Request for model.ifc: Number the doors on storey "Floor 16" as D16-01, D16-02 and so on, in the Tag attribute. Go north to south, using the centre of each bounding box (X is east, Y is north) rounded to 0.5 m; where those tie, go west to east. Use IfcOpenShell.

First a look at what the model holds.

```python
import ifcopenshell
import ifcopenshell.util.element
import ifcopenshell.util.placement

model = ifcopenshell.open("model.ifc")
print(model.schema)
storey = next(s for s in model.by_type("IfcBuildingStorey") if s.Name == "Floor 16")
doors = [e for e in ifcopenshell.util.element.get_decomposition(storey) if e.is_a("IfcDoor")]
for e in sorted(doors, key=lambda e: e.id()):
    origin = ifcopenshell.util.placement.get_local_placement(e.ObjectPlacement)[:3, 3]
    print(e.id(), e.Tag, e.Name, origin.round(2) + 0.0, sep=" | ")
```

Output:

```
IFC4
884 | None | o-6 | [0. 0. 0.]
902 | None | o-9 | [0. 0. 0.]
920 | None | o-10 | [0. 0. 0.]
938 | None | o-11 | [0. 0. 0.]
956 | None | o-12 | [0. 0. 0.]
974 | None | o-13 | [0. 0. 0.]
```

```python
import ifcopenshell
import ifcopenshell.geom
import ifcopenshell.util.element
import ifcopenshell.util.shape

model = ifcopenshell.open("model.ifc")
settings = ifcopenshell.geom.settings()
settings.set("use-world-coords", True)


def centre(element):
    shape = ifcopenshell.geom.create_shape(settings, element)
    return ifcopenshell.util.shape.get_bbox_centroid(shape.geometry)


storey = next(s for s in model.by_type("IfcBuildingStorey") if s.Name == "Floor 16")
doors = [e for e in ifcopenshell.util.element.get_decomposition(storey) if e.is_a("IfcDoor")]

# Insertion points can sit at a corner or the storey origin, so sort by the geometry (in metres).
centres = {e: centre(e) for e in doors}
doors.sort(key=lambda e: (-round(centres[e][1] / 0.5), centres[e][0]))

for i, e in enumerate(doors, start=1):
    number = f"D16-{i:02d}"
    e.Tag = number
    print(e.id(), number)

model.write("model_edited.ifc")
```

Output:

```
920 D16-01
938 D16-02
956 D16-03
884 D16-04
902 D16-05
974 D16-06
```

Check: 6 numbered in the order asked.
